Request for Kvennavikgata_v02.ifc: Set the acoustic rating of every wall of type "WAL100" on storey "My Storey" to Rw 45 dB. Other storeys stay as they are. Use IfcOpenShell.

First a look at what the model holds.

```python
import ifcopenshell
import ifcopenshell.util.element

model = ifcopenshell.open("Kvennavikgata_v02.ifc")
print(model.schema)
storey = next(s for s in model.by_type("IfcBuildingStorey") if s.Name == "My Storey")
walls = [e for e in ifcopenshell.util.element.get_decomposition(storey) if e.is_a("IfcWall")]
seen = {}
for e in walls:
    element_type = ifcopenshell.util.element.get_type(e)
    key = (element_type.Name if element_type != e and element_type else None, ifcopenshell.util.element.get_pset(e, "Pset_WallCommon", "AcousticRating"))
    seen[key] = seen.get(key, 0) + 1
for (name, value), count in sorted(seen.items(), key=str):
    print(count, "x", name, "|", value)
```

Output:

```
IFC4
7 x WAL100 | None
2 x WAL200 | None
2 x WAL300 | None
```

```python
import ifcopenshell
import ifcopenshell.api.pset
import ifcopenshell.util.element

model = ifcopenshell.open("Kvennavikgata_v02.ifc")

storey = next(s for s in model.by_type("IfcBuildingStorey") if s.Name == "My Storey")
walls = [e for e in ifcopenshell.util.element.get_decomposition(storey) if e.is_a("IfcWall")]

count = 0
for e in walls:
    element_type = ifcopenshell.util.element.get_type(e)
    if element_type in (None, e) or element_type.Name != "WAL100":
        continue
    # add_pset returns the element's existing set when there is one.
    pset = ifcopenshell.api.pset.add_pset(model, product=e, name="Pset_WallCommon")
    ifcopenshell.api.pset.edit_pset(model, pset=pset, properties={"AcousticRating": "Rw 45 dB"})
    count += 1

print(count, "walls updated")

model.write("Kvennavikgata_v02_v2.ifc")
```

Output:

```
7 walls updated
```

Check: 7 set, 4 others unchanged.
